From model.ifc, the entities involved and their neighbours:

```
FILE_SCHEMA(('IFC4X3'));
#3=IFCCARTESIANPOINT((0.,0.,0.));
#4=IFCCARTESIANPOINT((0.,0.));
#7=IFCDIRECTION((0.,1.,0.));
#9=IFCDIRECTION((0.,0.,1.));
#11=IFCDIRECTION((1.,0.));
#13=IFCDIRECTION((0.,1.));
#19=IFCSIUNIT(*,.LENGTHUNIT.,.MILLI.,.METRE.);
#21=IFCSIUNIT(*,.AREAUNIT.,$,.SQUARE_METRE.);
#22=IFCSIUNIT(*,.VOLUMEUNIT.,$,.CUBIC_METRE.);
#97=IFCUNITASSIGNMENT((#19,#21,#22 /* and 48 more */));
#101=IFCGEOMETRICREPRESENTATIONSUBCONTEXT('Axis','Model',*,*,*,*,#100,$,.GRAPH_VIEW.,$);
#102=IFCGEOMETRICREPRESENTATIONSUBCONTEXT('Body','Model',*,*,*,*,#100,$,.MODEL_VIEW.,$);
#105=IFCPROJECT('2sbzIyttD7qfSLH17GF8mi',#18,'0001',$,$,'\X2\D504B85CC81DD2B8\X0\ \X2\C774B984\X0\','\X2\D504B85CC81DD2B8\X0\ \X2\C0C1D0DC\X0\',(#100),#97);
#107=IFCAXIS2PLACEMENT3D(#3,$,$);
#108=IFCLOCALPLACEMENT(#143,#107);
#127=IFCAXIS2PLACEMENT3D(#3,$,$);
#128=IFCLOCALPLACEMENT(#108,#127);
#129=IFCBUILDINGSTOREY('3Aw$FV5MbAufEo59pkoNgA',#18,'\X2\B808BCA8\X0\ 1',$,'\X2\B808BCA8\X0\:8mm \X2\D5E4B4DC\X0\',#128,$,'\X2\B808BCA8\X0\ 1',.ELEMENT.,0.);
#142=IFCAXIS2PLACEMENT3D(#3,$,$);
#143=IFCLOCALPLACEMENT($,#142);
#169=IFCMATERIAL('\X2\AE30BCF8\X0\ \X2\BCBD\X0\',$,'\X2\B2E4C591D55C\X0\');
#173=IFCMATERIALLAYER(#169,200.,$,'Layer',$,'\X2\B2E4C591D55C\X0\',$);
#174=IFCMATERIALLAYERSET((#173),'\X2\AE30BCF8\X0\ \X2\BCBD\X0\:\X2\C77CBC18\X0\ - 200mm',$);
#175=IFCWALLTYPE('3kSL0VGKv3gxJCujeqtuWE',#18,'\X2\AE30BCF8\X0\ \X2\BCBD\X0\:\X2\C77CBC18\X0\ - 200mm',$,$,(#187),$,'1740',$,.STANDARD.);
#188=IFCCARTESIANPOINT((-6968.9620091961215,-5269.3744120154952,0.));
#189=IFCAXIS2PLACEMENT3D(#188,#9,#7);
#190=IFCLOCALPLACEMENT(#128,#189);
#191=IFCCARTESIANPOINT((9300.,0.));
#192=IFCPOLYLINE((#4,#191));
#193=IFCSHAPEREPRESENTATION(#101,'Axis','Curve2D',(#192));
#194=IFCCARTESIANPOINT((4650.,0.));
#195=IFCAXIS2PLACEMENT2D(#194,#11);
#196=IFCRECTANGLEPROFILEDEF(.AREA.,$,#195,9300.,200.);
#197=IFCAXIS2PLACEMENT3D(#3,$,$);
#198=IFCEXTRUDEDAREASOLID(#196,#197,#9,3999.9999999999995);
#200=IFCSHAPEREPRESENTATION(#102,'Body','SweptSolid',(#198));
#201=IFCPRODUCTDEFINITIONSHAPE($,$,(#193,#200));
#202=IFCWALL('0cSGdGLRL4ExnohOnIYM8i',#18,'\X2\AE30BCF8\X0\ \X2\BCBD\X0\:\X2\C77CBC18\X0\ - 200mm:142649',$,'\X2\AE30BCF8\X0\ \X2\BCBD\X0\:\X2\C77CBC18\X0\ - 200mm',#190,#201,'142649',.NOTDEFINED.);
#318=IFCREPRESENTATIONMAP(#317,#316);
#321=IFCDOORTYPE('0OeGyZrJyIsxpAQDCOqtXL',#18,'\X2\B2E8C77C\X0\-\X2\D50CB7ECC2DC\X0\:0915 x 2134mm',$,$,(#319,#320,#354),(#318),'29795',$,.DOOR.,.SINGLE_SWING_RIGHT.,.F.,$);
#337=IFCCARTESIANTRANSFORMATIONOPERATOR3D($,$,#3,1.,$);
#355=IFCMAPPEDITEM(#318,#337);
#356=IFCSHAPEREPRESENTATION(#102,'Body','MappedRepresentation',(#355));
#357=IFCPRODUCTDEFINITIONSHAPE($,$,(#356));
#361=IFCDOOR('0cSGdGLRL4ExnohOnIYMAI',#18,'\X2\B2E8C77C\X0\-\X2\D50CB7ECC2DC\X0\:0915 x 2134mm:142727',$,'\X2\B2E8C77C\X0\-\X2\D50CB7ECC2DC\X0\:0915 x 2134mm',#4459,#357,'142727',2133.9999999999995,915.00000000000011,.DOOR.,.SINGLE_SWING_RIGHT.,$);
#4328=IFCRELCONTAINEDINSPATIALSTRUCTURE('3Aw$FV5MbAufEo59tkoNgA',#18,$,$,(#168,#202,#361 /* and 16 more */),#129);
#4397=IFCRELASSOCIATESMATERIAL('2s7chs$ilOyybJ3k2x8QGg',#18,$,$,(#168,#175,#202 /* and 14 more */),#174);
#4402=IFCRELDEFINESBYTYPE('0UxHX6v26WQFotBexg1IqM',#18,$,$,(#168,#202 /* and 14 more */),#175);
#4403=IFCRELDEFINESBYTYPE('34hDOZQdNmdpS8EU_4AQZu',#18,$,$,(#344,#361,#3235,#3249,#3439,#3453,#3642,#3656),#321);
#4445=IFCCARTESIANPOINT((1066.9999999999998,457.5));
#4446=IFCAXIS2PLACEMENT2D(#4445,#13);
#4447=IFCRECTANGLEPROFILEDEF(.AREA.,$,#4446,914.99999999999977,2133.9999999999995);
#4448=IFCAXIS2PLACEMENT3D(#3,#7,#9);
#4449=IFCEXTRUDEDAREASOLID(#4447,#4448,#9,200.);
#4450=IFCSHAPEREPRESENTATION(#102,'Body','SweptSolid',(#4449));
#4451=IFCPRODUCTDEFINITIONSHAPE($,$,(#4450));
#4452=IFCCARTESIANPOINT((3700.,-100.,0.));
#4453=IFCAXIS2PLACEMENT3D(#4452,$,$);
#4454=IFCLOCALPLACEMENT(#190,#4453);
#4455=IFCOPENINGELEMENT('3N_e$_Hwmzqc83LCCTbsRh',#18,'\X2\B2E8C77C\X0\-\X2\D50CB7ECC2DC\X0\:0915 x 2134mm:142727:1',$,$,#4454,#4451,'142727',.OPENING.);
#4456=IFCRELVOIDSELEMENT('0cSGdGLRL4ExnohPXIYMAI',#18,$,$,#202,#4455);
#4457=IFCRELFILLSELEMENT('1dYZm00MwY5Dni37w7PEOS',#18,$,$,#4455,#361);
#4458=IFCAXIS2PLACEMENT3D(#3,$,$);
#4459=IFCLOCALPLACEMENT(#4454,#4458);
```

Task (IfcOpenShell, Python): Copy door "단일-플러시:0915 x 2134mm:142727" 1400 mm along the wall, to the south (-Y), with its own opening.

```python
import ifcopenshell
import ifcopenshell.api.feature
import ifcopenshell.api.geometry
import ifcopenshell.api.root
import ifcopenshell.geom
import ifcopenshell.util.element
import ifcopenshell.util.placement
import ifcopenshell.util.shape
import ifcopenshell.util.unit

model = ifcopenshell.open("model.ifc")
unit_scale = ifcopenshell.util.unit.calculate_unit_scale(model)
settings = ifcopenshell.geom.settings()


def volume(element):
    """Net volume in cubic metres, openings subtracted."""
    shape = ifcopenshell.geom.create_shape(settings, element)
    return ifcopenshell.util.shape.get_volume(shape.geometry)


def reuse_history(source, copy):
    """copy_class also copies each property set's owner history, people and application; keep the originals."""
    for rel in copy.IsDefinedBy:
        if rel.is_a("IfcRelDefinesByProperties") and (history := rel.RelatingPropertyDefinition.OwnerHistory):
            rel.RelatingPropertyDefinition.OwnerHistory = source.OwnerHistory
            ifcopenshell.util.element.remove_deep2(model, history)


door = model.by_id(361)
opening = door.FillsVoids[0].RelatingOpeningElement
wall = opening.VoidsElements[0].RelatingBuildingElement
before = volume(wall)
shift = ifcopenshell.util.placement.get_local_placement(wall.ObjectPlacement)[:3, 0] * -1.4 / unit_scale

# copy_class copies the void relationship, type, container and properties, but no geometry.
new_opening = ifcopenshell.api.root.copy_class(model, product=opening)
new_opening.Representation = ifcopenshell.util.element.copy_deep(
    model, opening.Representation, exclude=["IfcGeometricRepresentationContext", "IfcRepresentationMap"]
)
new_opening.Name = "단일-플러시:0915 x 2134mm"
new_opening.Tag = None
new_door = ifcopenshell.api.root.copy_class(model, product=door)
new_door.Representation = ifcopenshell.util.element.copy_deep(
    model, door.Representation, exclude=["IfcGeometricRepresentationContext", "IfcRepresentationMap"]
)
new_door.Name = "단일-플러시:0915 x 2134mm"
new_door.Tag = None
reuse_history(door, new_door)
ifcopenshell.api.feature.add_filling(model, opening=new_opening, element=new_door)

for old, new in ((opening, new_opening), (door, new_door)):
    matrix = ifcopenshell.util.placement.get_local_placement(old.ObjectPlacement)
    matrix[:3, 3] += shift
    ifcopenshell.api.geometry.edit_object_placement(model, product=new, matrix=matrix, is_si=False)

after = volume(wall)

print(f"wall volume {before:.3f} -> {after:.3f} m3")

model.write("model_v2.ifc")
```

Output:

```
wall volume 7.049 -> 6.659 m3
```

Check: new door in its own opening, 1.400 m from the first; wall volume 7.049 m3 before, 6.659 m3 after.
